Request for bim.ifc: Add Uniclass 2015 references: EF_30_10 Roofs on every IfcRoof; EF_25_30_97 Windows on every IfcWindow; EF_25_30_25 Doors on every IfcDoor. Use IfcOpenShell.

First a look at what the model holds.

```python
import ifcopenshell

model = ifcopenshell.open("bim.ifc")
print(model.schema)
print("classifications:", [c.Name for c in model.by_type("IfcClassification")])
for ifc_class in ("IfcDoor", "IfcRoof", "IfcStair", "IfcWall", "IfcWindow"):
    print(ifc_class, len(model.by_type(ifc_class)))
```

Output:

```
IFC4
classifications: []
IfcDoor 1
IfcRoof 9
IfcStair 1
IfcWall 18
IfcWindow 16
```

```python
import ifcopenshell
import ifcopenshell.api.classification

model = ifcopenshell.open("bim.ifc")

system = ifcopenshell.api.classification.add_classification(model, classification="Uniclass 2015")

codes = {
    "IfcRoof": ("EF_30_10", "Roofs"),
    "IfcWindow": ("EF_25_30_97", "Windows"),
    "IfcDoor": ("EF_25_30_25", "Doors"),
}
for ifc_class, (code, name) in codes.items():
    products = model.by_type(ifc_class)
    ifcopenshell.api.classification.add_reference(
        model, products=products, classification=system, identification=code, name=name
    )
    print(code, len(products))

model.write("bim_updated.ifc")
```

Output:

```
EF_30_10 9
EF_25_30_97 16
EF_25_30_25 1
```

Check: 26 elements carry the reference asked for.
